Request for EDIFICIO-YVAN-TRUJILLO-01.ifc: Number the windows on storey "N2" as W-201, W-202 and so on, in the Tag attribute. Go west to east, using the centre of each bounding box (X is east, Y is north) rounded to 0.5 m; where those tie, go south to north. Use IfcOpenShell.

First a look at what the model holds.

```python
import ifcopenshell
import ifcopenshell.util.element
import ifcopenshell.util.placement

model = ifcopenshell.open("EDIFICIO-YVAN-TRUJILLO-01.ifc")
print(model.schema)
storey = next(s for s in model.by_type("IfcBuildingStorey") if s.Name == "N2")
windows = [e for e in ifcopenshell.util.element.get_decomposition(storey) if e.is_a("IfcWindow")]
for e in sorted(windows, key=lambda e: e.id()):
    origin = ifcopenshell.util.placement.get_local_placement(e.ObjectPlacement)[:3, 3]
    print(e.id(), e.Tag, e.Name, origin.round(2) + 0.0, sep=" | ")
```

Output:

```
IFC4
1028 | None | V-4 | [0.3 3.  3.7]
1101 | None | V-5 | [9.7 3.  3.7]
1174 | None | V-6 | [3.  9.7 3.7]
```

```python
import ifcopenshell
import ifcopenshell.geom
import ifcopenshell.util.element
import ifcopenshell.util.shape

model = ifcopenshell.open("EDIFICIO-YVAN-TRUJILLO-01.ifc")
settings = ifcopenshell.geom.settings()
settings.set("use-world-coords", True)


def centre(element):
    shape = ifcopenshell.geom.create_shape(settings, element)
    return ifcopenshell.util.shape.get_bbox_centroid(shape.geometry)


storey = next(s for s in model.by_type("IfcBuildingStorey") if s.Name == "N2")
windows = [e for e in ifcopenshell.util.element.get_decomposition(storey) if e.is_a("IfcWindow")]

# Insertion points can sit at a corner or the storey origin, so sort by the geometry (in metres).
centres = {e: centre(e) for e in windows}
windows.sort(key=lambda e: (round(centres[e][0] / 0.5), centres[e][1]))

for i, e in enumerate(windows, start=1):
    number = f"W-2{i:02d}"
    e.Tag = number
    print(e.id(), number)

model.write("EDIFICIO-YVAN-TRUJILLO-01_rev.ifc")
```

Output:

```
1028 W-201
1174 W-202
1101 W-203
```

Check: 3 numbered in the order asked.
